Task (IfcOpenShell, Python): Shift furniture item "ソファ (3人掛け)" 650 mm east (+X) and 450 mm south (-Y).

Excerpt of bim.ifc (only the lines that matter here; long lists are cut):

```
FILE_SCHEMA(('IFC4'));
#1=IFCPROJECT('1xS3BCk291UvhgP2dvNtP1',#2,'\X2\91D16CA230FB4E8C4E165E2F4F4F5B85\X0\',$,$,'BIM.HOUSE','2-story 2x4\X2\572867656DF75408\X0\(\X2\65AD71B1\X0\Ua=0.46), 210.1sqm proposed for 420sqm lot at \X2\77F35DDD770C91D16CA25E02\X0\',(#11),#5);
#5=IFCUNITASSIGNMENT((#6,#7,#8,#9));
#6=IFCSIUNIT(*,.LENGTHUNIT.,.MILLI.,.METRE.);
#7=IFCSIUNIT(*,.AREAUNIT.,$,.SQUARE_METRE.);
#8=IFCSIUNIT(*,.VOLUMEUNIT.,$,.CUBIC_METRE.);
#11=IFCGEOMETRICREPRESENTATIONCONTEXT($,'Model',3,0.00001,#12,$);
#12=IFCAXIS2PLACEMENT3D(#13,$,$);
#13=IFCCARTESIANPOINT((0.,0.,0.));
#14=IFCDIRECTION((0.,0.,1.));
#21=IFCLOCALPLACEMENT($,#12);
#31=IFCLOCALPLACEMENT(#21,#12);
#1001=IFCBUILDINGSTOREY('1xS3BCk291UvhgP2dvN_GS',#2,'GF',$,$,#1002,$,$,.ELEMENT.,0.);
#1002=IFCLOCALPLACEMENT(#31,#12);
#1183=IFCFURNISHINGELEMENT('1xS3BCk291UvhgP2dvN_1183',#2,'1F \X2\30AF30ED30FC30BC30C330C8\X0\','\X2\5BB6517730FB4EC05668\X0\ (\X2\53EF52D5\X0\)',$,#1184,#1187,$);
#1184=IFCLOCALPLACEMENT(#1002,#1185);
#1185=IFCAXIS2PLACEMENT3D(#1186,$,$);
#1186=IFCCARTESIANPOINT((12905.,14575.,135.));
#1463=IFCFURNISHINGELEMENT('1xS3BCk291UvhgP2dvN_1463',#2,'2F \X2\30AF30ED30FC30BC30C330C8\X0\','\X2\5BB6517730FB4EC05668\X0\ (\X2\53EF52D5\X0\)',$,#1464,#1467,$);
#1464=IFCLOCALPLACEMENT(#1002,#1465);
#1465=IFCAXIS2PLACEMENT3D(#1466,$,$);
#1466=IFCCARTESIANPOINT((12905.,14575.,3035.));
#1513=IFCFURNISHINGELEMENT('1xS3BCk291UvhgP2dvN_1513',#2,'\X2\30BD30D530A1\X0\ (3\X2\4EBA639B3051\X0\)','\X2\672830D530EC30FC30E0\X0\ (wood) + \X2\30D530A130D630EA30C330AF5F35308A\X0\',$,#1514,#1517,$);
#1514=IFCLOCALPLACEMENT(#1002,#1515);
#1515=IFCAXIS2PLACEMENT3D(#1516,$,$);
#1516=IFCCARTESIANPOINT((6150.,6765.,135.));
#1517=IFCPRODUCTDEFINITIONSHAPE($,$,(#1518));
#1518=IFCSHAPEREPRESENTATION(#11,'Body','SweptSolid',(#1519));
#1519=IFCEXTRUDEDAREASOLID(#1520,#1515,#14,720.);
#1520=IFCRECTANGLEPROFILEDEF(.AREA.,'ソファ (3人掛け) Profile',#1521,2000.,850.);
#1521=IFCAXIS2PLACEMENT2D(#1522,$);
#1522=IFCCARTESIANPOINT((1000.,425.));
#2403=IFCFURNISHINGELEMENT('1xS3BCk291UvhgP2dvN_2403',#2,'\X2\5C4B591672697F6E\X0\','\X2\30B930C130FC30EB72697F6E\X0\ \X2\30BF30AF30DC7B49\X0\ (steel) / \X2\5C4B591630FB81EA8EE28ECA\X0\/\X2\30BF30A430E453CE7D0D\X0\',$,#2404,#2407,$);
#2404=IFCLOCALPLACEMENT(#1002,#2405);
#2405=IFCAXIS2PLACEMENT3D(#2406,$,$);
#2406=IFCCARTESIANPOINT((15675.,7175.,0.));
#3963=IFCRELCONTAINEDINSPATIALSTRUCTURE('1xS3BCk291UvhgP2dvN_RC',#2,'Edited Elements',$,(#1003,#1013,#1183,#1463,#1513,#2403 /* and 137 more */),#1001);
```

```python
import ifcopenshell
import ifcopenshell.api.geometry
import ifcopenshell.util.placement

model = ifcopenshell.open("bim.ifc")

item = model.by_id(1513)
matrix = ifcopenshell.util.placement.get_local_placement(item.ObjectPlacement)
matrix[0, 3] += 650.0
matrix[1, 3] -= 450.0
ifcopenshell.api.geometry.edit_object_placement(model, product=item, matrix=matrix, is_si=False)

print(ifcopenshell.util.placement.get_local_placement(item.ObjectPlacement).round(3) + 0.0)

model.write("bim_updated.ifc")
```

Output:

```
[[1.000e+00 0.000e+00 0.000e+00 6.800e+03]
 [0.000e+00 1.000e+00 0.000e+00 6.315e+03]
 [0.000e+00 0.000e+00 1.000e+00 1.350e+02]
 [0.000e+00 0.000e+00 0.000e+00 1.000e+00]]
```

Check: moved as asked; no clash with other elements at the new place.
